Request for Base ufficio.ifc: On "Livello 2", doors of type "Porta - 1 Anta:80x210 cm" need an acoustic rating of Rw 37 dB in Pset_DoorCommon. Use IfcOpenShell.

First a look at what the model holds.

```python
import ifcopenshell
import ifcopenshell.util.element

model = ifcopenshell.open("Base ufficio.ifc")
print(model.schema)
storey = next(s for s in model.by_type("IfcBuildingStorey") if s.Name == "Livello 2")
doors = [e for e in ifcopenshell.util.element.get_decomposition(storey) if e.is_a("IfcDoor")]
seen = {}
for e in doors:
    element_type = ifcopenshell.util.element.get_type(e)
    key = (element_type.Name if element_type != e and element_type else None, ifcopenshell.util.element.get_pset(e, "Pset_DoorCommon", "AcousticRating"))
    seen[key] = seen.get(key, 0) + 1
for (name, value), count in sorted(seen.items(), key=str):
    print(count, "x", name, "|", value)
```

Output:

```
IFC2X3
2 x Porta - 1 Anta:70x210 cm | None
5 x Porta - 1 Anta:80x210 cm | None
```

```python
import ifcopenshell
import ifcopenshell.api.pset
import ifcopenshell.util.element

model = ifcopenshell.open("Base ufficio.ifc")

storey = next(s for s in model.by_type("IfcBuildingStorey") if s.Name == "Livello 2")
doors = [e for e in ifcopenshell.util.element.get_decomposition(storey) if e.is_a("IfcDoor")]

count = 0
for e in doors:
    element_type = ifcopenshell.util.element.get_type(e)
    if element_type in (None, e) or element_type.Name != "Porta - 1 Anta:80x210 cm":
        continue
    # add_pset returns the element's existing set when there is one.
    pset = ifcopenshell.api.pset.add_pset(model, product=e, name="Pset_DoorCommon")
    ifcopenshell.api.pset.edit_pset(model, pset=pset, properties={"AcousticRating": "Rw 37 dB"})
    count += 1

print(count, "doors updated")

model.write("Base ufficio_edited.ifc")
```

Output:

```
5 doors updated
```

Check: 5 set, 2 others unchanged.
